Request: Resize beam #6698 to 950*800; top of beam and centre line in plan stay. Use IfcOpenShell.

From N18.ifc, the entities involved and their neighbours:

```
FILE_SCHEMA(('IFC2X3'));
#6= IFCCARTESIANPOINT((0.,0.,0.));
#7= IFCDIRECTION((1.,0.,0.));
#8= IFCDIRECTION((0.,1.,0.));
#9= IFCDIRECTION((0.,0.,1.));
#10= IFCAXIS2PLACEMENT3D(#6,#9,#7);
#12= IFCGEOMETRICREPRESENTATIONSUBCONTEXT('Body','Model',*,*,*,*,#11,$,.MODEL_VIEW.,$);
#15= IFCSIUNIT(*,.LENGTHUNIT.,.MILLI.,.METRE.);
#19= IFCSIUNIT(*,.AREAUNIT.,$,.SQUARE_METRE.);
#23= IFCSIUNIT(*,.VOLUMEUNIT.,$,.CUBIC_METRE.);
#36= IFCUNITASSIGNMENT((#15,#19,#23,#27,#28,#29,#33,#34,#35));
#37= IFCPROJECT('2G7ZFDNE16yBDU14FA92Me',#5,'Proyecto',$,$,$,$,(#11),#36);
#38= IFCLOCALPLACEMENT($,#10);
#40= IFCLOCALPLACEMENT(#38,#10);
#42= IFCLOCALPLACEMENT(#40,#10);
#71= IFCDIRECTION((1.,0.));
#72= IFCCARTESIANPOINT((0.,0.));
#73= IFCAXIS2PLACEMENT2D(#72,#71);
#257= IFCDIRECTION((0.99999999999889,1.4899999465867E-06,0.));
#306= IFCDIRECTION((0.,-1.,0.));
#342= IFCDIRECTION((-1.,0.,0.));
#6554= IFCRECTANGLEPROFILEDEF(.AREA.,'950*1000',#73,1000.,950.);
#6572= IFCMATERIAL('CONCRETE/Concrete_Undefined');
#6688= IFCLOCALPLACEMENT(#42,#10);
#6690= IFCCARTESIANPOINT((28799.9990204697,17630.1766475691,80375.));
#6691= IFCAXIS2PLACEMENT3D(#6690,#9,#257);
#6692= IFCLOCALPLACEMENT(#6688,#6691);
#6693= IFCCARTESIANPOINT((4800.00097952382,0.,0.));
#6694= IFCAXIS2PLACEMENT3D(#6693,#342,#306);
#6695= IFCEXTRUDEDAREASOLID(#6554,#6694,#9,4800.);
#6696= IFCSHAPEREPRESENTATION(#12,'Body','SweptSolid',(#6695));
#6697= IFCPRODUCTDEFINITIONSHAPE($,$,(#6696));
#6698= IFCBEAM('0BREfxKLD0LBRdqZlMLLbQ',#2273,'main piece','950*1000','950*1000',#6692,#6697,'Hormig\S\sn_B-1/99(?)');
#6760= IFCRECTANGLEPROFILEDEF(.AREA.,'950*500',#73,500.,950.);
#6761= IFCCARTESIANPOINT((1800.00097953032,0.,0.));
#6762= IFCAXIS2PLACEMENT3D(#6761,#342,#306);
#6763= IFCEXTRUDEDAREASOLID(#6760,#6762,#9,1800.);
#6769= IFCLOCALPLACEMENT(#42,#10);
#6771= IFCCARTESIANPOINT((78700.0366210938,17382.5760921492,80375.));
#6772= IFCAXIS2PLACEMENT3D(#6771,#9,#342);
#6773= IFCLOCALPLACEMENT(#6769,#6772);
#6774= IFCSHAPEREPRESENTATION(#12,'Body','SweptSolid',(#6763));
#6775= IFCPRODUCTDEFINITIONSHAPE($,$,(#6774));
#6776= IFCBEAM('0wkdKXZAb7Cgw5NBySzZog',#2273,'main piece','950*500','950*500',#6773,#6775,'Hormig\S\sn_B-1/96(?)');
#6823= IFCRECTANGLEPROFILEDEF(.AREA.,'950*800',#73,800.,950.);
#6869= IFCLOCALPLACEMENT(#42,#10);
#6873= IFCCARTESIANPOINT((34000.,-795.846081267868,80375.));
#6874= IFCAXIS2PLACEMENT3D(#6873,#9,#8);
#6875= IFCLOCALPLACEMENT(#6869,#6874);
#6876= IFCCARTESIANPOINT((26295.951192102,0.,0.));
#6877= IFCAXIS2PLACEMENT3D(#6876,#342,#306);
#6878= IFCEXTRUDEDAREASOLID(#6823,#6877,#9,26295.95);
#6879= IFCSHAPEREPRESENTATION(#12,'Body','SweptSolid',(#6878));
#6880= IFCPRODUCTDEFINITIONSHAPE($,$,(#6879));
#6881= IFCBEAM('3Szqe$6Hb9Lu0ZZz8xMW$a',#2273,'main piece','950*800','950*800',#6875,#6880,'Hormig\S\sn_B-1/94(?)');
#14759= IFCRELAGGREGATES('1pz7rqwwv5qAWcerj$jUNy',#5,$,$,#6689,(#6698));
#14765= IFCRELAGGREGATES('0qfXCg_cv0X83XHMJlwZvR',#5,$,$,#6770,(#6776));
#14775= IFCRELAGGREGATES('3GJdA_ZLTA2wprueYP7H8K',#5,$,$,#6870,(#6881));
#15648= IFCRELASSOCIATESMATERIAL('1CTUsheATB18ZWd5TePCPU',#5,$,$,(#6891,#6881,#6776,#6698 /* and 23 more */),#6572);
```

```python
import ifcopenshell
import ifcopenshell.util.element
import ifcopenshell.util.representation

model = ifcopenshell.open("N18.ifc")

member = model.by_guid("0BREfxKLD0LBRdqZlMLLbQ")
source = next(p for p in model.by_type("IfcRectangleProfileDef") if p.ProfileName == "950*800")

body = ifcopenshell.util.representation.get_representation(member, "Model", "Body")
solid = body.Items[0]
old_profile = solid.SweptArea

# Copy the section's sizes but keep this member's own profile position.
profile = ifcopenshell.util.element.copy(model, source)
# Profiles are centred, so shift by half the change in depth to hold the top.
shift = (old_profile.YDim - profile.YDim) / 2
x, y = old_profile.Position.Location.Coordinates
up = (0.0, 1.0)  # upwards, in the solid's own plane
location = model.createIfcCartesianPoint((x + up[0] * shift, y + up[1] * shift))
profile.Position = model.createIfcAxis2Placement2D(location, old_profile.Position.RefDirection)
solid.SweptArea = profile
if not model.get_total_inverses(old_profile):
    ifcopenshell.util.element.remove_deep2(model, old_profile)
member.Description = member.Description.replace("950*1000", "950*800")
member.ObjectType = member.ObjectType.replace("950*1000", "950*800")

print(solid.SweptArea)

model.write("N18_updated.ifc")
```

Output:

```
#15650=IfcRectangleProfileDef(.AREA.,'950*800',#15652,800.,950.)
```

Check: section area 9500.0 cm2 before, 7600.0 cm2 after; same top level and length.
